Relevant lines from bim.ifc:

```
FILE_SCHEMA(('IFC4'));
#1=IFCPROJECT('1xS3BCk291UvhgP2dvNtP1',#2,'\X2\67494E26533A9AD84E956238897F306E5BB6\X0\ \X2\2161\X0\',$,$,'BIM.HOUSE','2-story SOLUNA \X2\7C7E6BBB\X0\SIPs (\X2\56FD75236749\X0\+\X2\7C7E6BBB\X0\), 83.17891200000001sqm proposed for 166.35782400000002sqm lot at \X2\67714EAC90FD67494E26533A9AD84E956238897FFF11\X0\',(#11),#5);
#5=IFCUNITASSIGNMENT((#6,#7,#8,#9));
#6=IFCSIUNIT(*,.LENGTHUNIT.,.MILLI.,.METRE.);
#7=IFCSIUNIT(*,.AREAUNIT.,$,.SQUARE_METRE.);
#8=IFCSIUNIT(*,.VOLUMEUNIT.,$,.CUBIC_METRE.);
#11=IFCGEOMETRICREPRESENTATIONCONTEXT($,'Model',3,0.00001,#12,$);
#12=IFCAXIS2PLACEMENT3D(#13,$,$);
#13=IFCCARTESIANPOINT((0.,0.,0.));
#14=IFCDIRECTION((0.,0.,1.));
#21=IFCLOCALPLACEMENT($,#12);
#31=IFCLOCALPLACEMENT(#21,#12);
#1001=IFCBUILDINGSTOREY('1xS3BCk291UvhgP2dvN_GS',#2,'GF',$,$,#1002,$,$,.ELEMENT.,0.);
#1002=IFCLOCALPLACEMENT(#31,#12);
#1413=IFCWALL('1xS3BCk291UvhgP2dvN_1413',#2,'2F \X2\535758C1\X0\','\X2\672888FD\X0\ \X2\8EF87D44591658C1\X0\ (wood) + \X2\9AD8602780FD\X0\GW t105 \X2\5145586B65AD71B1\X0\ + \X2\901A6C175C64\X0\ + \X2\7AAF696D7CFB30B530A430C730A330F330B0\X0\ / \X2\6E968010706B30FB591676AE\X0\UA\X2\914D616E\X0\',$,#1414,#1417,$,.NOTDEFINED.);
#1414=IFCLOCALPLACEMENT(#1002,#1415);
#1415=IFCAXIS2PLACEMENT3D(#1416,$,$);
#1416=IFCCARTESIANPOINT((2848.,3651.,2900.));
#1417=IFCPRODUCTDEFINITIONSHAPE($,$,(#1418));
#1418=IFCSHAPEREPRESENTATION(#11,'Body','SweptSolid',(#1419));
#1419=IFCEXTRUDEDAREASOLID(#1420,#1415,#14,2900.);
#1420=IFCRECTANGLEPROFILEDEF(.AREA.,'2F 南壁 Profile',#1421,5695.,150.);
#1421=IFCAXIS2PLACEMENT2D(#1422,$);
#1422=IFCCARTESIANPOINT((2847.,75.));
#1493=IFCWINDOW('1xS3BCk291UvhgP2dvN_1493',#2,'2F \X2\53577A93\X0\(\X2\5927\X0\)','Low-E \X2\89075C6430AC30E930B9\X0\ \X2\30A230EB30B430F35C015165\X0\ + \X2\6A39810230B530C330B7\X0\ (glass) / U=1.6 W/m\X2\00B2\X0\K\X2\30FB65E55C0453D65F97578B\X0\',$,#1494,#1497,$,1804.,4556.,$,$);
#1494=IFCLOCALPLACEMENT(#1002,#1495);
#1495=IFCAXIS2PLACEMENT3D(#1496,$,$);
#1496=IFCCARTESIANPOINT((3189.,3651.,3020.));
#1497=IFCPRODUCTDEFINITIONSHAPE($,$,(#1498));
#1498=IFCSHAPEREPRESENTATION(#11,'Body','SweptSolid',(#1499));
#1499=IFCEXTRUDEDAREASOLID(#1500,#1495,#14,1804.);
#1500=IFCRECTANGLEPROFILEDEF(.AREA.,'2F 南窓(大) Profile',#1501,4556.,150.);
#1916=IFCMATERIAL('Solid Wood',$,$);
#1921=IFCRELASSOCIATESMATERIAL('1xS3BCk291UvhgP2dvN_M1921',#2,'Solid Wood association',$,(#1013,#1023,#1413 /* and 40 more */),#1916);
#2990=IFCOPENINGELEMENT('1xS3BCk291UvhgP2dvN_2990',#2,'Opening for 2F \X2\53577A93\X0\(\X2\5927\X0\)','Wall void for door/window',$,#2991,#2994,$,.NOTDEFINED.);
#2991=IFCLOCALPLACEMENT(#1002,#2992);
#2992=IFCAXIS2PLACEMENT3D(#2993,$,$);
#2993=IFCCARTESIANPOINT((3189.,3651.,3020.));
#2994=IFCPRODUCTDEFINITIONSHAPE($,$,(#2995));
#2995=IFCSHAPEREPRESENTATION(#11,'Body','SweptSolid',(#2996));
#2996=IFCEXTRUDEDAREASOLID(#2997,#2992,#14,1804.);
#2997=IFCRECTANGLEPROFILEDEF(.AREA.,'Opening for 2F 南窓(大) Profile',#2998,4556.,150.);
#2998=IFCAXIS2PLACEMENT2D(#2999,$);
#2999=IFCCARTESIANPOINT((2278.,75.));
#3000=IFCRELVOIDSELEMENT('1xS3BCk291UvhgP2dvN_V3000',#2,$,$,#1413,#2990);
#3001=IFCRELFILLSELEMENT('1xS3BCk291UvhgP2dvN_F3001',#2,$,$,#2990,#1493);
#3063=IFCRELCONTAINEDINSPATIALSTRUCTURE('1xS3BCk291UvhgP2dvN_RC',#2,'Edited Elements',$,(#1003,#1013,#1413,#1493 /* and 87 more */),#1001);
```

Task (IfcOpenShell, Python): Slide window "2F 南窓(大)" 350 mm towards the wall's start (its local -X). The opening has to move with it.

```python
import ifcopenshell
import ifcopenshell.api.geometry
import ifcopenshell.util.placement
import ifcopenshell.util.unit

model = ifcopenshell.open("bim.ifc")
unit_scale = ifcopenshell.util.unit.calculate_unit_scale(model)

window = model.by_guid("1xS3BCk291UvhgP2dvN_1493")
opening = window.FillsVoids[0].RelatingOpeningElement
wall = opening.VoidsElements[0].RelatingBuildingElement

wall_matrix = ifcopenshell.util.placement.get_local_placement(wall.ObjectPlacement)
shift = wall_matrix[:3, 0] * -0.35 / unit_scale
before = ifcopenshell.util.placement.get_local_placement(window.ObjectPlacement)[:3, 3].copy()

# The window is not placed relative to its opening, so move both.
for product in (opening, window):
    matrix = ifcopenshell.util.placement.get_local_placement(product.ObjectPlacement)
    matrix[:3, 3] += shift
    ifcopenshell.api.geometry.edit_object_placement(model, product=product, matrix=matrix, is_si=False)

after = ifcopenshell.util.placement.get_local_placement(window.ObjectPlacement)[:3, 3]
print("window moved by", (after - before).round(3) + 0.0)

model.write("bim_rev.ifc")
```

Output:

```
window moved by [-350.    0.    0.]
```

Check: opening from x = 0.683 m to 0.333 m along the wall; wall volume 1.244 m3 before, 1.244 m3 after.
